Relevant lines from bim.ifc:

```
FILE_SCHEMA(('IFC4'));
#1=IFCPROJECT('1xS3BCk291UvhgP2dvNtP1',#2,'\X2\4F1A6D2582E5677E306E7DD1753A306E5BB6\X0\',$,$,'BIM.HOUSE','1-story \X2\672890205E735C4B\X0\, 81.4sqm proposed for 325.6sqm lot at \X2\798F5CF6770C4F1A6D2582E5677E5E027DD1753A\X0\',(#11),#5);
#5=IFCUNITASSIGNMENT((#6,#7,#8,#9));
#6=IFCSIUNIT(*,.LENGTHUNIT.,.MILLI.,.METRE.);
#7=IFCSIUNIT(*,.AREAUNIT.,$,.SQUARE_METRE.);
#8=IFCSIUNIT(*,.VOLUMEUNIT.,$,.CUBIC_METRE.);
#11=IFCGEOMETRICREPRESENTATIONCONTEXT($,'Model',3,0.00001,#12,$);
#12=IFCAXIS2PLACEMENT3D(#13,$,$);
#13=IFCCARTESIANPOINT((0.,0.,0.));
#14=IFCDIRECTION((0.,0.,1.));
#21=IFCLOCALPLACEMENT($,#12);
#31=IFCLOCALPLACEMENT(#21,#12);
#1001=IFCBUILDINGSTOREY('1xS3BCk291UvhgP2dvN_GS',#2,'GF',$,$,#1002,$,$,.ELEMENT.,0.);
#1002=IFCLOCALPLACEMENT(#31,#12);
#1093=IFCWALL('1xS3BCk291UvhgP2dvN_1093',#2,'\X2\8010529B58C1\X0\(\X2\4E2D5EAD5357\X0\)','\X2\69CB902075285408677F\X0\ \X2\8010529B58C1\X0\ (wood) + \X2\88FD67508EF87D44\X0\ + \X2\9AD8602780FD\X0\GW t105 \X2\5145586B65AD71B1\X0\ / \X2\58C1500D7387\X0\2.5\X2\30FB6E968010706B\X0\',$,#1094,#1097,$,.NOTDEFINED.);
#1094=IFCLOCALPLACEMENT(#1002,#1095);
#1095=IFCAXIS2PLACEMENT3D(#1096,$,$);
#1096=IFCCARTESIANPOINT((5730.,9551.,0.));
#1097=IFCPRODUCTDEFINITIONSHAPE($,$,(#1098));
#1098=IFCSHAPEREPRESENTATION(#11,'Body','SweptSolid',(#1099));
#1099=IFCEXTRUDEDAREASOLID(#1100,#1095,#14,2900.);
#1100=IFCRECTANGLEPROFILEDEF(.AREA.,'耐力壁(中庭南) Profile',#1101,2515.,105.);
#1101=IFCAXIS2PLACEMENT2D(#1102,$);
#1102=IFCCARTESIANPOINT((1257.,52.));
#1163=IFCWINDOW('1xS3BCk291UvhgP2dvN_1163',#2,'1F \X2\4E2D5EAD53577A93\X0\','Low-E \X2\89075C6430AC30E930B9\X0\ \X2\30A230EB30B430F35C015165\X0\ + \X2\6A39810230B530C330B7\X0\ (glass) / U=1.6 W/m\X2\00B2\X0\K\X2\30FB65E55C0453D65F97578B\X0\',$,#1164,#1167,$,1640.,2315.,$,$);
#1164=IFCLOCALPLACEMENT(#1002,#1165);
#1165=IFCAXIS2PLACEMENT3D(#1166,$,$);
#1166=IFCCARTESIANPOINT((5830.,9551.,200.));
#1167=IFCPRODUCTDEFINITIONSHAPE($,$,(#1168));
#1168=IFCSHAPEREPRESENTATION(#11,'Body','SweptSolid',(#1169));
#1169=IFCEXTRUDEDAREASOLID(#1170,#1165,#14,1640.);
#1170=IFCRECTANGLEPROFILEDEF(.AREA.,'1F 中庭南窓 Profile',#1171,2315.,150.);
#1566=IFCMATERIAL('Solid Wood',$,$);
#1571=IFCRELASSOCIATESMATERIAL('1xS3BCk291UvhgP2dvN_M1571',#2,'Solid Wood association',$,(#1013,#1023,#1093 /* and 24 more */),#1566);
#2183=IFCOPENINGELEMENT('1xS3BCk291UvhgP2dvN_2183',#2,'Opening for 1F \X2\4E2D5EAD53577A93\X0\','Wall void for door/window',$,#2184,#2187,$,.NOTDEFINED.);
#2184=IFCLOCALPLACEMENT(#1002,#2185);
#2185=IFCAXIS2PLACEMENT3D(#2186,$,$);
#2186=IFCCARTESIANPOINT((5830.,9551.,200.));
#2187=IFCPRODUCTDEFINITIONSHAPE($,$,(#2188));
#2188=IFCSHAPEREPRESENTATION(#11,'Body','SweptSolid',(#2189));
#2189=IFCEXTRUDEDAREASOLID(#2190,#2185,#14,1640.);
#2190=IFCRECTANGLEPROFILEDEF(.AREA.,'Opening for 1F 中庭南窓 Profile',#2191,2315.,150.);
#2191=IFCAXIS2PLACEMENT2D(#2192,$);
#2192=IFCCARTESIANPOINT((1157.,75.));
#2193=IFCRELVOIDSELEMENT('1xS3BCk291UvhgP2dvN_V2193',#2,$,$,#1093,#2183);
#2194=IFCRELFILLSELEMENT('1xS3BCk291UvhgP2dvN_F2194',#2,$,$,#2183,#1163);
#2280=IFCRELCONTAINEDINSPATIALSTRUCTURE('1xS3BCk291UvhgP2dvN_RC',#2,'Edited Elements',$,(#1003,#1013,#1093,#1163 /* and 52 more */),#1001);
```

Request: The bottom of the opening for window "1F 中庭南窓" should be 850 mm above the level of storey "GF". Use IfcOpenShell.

```python
import numpy as np
import ifcopenshell
import ifcopenshell.api.geometry
import ifcopenshell.geom
import ifcopenshell.util.element
import ifcopenshell.util.placement
import ifcopenshell.util.shape
import ifcopenshell.util.unit

model = ifcopenshell.open("bim.ifc")
unit_scale = ifcopenshell.util.unit.calculate_unit_scale(model)

window = model.by_id(1163)
opening = window.FillsVoids[0].RelatingOpeningElement
storey = ifcopenshell.util.element.get_container(window, ifc_class="IfcBuildingStorey")
level = ifcopenshell.util.placement.get_local_placement(storey.ObjectPlacement)[2, 3]

# The opening's origin need not be at the sill, so measure its lowest point.
shape = ifcopenshell.geom.create_shape(ifcopenshell.geom.settings(), opening)
bottom = ifcopenshell.util.shape.get_shape_bottom_elevation(shape, shape.geometry) / unit_scale
dz = level + 0.85 / unit_scale - bottom

shift = np.array([0.0, 0.0, dz])
# The window is not placed relative to its opening, so move both.
for product in (opening, window):
    matrix = ifcopenshell.util.placement.get_local_placement(product.ObjectPlacement)
    matrix[:3, 3] += shift
    ifcopenshell.api.geometry.edit_object_placement(model, product=product, matrix=matrix, is_si=False)

print(f"moved by {dz * unit_scale:+.3f} m")

model.write("bim_edited.ifc")
```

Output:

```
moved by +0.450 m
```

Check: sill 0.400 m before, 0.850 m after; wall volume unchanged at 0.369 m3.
